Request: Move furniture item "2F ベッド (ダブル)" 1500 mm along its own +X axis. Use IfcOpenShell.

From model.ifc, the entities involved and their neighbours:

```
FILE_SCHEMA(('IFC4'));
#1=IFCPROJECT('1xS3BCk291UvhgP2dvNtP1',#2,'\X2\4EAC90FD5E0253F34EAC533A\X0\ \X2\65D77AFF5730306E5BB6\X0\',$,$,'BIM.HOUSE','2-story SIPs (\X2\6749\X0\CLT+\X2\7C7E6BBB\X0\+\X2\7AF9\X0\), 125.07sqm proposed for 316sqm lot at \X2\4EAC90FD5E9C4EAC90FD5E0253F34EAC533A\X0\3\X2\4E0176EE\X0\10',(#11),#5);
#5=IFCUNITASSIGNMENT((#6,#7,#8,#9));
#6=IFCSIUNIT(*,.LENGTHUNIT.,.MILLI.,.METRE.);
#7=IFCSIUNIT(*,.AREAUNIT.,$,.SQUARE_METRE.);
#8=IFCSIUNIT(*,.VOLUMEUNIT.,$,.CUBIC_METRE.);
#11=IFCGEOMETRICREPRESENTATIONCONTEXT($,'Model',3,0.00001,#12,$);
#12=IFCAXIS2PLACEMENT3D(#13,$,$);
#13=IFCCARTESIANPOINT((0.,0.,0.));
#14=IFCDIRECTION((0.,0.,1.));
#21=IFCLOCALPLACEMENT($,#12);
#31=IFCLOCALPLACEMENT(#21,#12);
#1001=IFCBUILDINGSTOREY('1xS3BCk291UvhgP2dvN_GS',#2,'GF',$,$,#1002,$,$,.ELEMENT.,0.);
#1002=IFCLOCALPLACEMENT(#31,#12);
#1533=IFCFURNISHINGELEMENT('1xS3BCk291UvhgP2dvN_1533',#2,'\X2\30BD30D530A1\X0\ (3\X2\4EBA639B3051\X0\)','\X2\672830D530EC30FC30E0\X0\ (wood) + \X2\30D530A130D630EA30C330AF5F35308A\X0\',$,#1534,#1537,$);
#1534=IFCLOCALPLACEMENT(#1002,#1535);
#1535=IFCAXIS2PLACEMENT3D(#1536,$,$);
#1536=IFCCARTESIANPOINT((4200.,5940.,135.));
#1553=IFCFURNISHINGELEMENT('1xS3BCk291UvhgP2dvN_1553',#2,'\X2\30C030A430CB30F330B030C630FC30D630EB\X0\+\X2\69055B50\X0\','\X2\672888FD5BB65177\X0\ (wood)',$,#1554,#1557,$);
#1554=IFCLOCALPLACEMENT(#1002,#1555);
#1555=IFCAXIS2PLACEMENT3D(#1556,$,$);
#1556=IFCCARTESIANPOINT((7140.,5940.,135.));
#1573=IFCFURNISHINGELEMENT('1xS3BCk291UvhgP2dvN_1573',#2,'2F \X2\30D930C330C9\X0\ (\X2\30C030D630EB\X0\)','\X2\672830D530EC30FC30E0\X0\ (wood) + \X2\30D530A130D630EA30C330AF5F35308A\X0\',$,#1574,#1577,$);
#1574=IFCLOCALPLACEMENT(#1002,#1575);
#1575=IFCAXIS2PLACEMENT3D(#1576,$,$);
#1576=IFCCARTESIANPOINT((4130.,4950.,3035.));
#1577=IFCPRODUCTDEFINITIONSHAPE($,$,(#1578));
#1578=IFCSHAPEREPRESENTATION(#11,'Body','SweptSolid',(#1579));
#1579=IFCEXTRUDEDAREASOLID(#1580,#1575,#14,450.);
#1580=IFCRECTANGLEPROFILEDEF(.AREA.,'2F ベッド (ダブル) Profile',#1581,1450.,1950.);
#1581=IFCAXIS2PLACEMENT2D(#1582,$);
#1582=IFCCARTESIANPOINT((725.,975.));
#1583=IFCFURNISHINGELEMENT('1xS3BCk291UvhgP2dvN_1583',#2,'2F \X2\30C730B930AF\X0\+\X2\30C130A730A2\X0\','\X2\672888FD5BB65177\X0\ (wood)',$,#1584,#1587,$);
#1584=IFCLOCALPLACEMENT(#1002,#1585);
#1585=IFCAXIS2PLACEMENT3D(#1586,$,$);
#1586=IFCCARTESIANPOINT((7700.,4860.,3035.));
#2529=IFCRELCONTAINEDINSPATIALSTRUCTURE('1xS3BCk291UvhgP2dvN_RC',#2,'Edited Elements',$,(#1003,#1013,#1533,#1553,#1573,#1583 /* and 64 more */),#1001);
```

```python
import ifcopenshell
import ifcopenshell.api.geometry
import ifcopenshell.util.placement

model = ifcopenshell.open("model.ifc")

item = model.by_guid("1xS3BCk291UvhgP2dvN_1573")
matrix = ifcopenshell.util.placement.get_local_placement(item.ObjectPlacement)
matrix[:3, 3] += matrix[:3, 0] * 1500.0
ifcopenshell.api.geometry.edit_object_placement(model, product=item, matrix=matrix, is_si=False)

print(ifcopenshell.util.placement.get_local_placement(item.ObjectPlacement).round(3) + 0.0)

model.write("model_edited.ifc")
```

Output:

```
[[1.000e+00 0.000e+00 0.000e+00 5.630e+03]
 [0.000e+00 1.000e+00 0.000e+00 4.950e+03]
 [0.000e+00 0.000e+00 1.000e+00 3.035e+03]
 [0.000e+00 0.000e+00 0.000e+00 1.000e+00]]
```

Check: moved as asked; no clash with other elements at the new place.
